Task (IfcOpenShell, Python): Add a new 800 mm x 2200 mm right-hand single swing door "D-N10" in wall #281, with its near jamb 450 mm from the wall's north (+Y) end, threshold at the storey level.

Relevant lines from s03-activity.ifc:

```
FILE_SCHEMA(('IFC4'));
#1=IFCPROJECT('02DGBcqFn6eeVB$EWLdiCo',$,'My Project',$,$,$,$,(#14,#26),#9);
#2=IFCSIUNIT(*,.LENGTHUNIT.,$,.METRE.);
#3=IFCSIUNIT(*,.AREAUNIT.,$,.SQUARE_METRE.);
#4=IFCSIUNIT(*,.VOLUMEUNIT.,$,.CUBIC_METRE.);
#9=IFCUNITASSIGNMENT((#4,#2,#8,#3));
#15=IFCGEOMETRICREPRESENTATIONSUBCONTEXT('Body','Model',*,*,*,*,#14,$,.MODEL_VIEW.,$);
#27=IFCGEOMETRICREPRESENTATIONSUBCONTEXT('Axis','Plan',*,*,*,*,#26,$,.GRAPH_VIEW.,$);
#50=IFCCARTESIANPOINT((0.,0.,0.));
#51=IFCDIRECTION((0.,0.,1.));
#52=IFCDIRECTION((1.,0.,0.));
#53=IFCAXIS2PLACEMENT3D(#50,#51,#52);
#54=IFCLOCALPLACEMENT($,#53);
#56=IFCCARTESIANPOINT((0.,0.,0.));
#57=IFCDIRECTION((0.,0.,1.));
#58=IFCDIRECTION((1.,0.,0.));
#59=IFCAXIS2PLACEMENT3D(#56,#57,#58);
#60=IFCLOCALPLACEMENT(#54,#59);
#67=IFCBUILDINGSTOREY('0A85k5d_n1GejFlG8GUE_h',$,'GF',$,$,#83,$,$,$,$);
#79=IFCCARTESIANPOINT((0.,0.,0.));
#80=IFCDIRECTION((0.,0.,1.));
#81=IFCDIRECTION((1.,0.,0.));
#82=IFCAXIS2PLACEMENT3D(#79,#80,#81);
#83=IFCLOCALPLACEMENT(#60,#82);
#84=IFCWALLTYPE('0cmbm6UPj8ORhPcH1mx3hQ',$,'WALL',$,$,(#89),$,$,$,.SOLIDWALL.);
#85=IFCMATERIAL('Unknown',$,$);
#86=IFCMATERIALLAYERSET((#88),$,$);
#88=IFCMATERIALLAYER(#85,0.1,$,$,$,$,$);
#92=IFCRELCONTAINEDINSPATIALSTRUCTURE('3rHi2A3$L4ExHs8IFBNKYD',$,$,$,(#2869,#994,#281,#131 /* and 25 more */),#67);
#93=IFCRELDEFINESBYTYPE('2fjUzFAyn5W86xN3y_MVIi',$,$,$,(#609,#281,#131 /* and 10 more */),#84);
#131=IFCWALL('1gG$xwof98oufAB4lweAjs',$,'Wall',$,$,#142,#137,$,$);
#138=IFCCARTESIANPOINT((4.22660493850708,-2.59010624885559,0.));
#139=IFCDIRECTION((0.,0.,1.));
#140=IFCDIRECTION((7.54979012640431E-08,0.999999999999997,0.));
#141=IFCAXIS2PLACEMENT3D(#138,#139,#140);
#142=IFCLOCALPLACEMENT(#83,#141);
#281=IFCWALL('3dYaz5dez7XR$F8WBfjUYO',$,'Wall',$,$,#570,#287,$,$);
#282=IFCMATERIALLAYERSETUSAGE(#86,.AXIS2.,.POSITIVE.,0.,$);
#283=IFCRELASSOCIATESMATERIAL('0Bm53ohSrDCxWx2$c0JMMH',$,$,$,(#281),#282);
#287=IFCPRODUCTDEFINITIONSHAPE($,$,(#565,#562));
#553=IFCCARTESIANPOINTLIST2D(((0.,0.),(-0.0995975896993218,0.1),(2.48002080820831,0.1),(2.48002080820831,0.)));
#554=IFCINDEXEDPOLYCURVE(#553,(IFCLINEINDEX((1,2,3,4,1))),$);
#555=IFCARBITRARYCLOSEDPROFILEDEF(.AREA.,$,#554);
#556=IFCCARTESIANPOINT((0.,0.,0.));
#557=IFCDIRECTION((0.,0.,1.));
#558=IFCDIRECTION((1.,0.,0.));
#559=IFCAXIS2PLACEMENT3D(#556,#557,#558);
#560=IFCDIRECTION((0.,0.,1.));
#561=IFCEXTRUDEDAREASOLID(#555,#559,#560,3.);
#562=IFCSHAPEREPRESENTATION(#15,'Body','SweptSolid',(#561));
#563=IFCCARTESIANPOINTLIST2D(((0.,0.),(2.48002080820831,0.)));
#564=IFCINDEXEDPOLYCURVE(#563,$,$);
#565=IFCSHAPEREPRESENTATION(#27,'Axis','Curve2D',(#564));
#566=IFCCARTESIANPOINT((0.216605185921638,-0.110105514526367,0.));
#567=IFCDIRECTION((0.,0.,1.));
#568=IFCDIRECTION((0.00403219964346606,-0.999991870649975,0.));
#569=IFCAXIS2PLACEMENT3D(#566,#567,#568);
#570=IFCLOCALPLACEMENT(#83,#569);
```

```python
import numpy as np
import ifcopenshell
import ifcopenshell.api.feature
import ifcopenshell.api.geometry
import ifcopenshell.api.root
import ifcopenshell.api.spatial
import ifcopenshell.geom
import ifcopenshell.util.element
import ifcopenshell.util.placement
import ifcopenshell.util.representation
import ifcopenshell.util.shape
import ifcopenshell.util.unit

model = ifcopenshell.open("s03-activity.ifc")
unit_scale = ifcopenshell.util.unit.calculate_unit_scale(model)
settings = ifcopenshell.geom.settings()


def volume(element):
    """Net volume in cubic metres, openings subtracted."""
    shape = ifcopenshell.geom.create_shape(settings, element)
    return ifcopenshell.util.shape.get_volume(shape.geometry)


wall = model.by_guid("3dYaz5dez7XR$F8WBfjUYO")
storey = ifcopenshell.util.element.get_container(wall, ifc_class="IfcBuildingStorey")
context = ifcopenshell.util.representation.get_context(model, "Model", "Body", "MODEL_VIEW")
before = volume(wall)

width, height, from_end, sill = 0.8, 2.2, 0.45, 0.0  # metres

# The wall runs along its own X axis, and the end named is its -X end.
wall_shape = ifcopenshell.geom.create_shape(settings, wall)
x, y, z = ifcopenshell.util.shape.get_vertices(wall_shape.geometry).T
start = x.min() + from_end
face, thickness = float(y.min()), float(y.max() - y.min())
wall_matrix = ifcopenshell.util.placement.get_local_placement(wall.ObjectPlacement)
level = ifcopenshell.util.placement.get_local_placement(storey.ObjectPlacement)[2, 3]


def in_wall(x, y):
    """Placement at x, y metres in the wall's axes, at sill height."""
    matrix = wall_matrix.copy()
    matrix[:, 3] = wall_matrix @ np.array([x / unit_scale, y / unit_scale, 0.0, 1.0])
    matrix[2, 3] = level + sill / unit_scale
    return matrix


# Opening: a box that overshoots both wall faces by 50 mm.
opening = ifcopenshell.api.root.create_entity(model, ifc_class="IfcOpeningElement", predefined_type="OPENING")
box = ifcopenshell.api.geometry.add_wall_representation(
    model, context=context, length=width, height=height, thickness=thickness + 0.1
)
ifcopenshell.api.geometry.assign_representation(model, product=opening, representation=box)
ifcopenshell.api.geometry.edit_object_placement(model, product=opening, matrix=in_wall(start, face - 0.05), is_si=False)
ifcopenshell.api.feature.add_feature(model, feature=opening, element=wall)

door = ifcopenshell.api.root.create_entity(model, ifc_class="IfcDoor", name="D-N10", predefined_type="DOOR")
door.OverallWidth, door.OverallHeight = width / unit_scale, height / unit_scale
door.OperationType = "SINGLE_SWING_RIGHT"
body = ifcopenshell.api.geometry.add_door_representation(
    model,
    context=context,
    overall_width=door.OverallWidth,
    overall_height=door.OverallHeight,
    operation_type="SINGLE_SWING_RIGHT",
    lining_properties={"LiningDepth": thickness / unit_scale, "ThresholdDepth": thickness / unit_scale},
)
ifcopenshell.api.geometry.assign_representation(model, product=door, representation=body)
ifcopenshell.api.spatial.assign_container(model, products=[door], relating_structure=storey)
ifcopenshell.api.feature.add_filling(model, opening=opening, element=door)

# The lining spans the wall, so the door starts at the wall face.
ifcopenshell.api.geometry.edit_object_placement(model, product=door, matrix=in_wall(start, face), is_si=False)

after = volume(wall)

print(f"wall volume {before:.3f} -> {after:.3f} m3")

model.write("s03-activity-out.ifc")
```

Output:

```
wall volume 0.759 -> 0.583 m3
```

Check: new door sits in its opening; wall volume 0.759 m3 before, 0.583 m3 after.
